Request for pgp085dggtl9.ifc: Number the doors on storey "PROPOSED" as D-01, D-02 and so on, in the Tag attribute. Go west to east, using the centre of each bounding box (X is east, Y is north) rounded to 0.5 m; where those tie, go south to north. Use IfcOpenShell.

First a look at what the model holds.

```python
import ifcopenshell
import ifcopenshell.util.element
import ifcopenshell.util.placement

model = ifcopenshell.open("pgp085dggtl9.ifc")
print(model.schema)
storey = next(s for s in model.by_type("IfcBuildingStorey") if s.Name == "PROPOSED")
doors = [e for e in ifcopenshell.util.element.get_decomposition(storey) if e.is_a("IfcDoor")]
for e in sorted(doors, key=lambda e: e.id()):
    origin = ifcopenshell.util.placement.get_local_placement(e.ObjectPlacement)[:3, 3]
    print(e.id(), e.Tag, e.Name, origin.round(2) + 0.0, sep=" | ")
```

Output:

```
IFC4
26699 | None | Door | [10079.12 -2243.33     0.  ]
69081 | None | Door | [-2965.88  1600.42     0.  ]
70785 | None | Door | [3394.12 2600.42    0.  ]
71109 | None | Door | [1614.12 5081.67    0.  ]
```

```python
import ifcopenshell
import ifcopenshell.geom
import ifcopenshell.util.element
import ifcopenshell.util.shape

model = ifcopenshell.open("pgp085dggtl9.ifc")
settings = ifcopenshell.geom.settings()
settings.set("use-world-coords", True)


def centre(element):
    shape = ifcopenshell.geom.create_shape(settings, element)
    return ifcopenshell.util.shape.get_bbox_centroid(shape.geometry)


storey = next(s for s in model.by_type("IfcBuildingStorey") if s.Name == "PROPOSED")
doors = [e for e in ifcopenshell.util.element.get_decomposition(storey) if e.is_a("IfcDoor")]

# Insertion points can sit at a corner or the storey origin, so sort by the geometry (in metres).
centres = {e: centre(e) for e in doors}
doors.sort(key=lambda e: (round(centres[e][0] / 0.5), centres[e][1]))

for i, e in enumerate(doors, start=1):
    number = f"D-{i:02d}"
    e.Tag = number
    print(e.id(), number)

model.write("pgp085dggtl9_v2.ifc")
```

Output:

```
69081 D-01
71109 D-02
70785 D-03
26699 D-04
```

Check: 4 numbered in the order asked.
